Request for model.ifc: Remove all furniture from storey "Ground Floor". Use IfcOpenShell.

First a look at what the model holds.

```python
import ifcopenshell
import ifcopenshell.util.element

model = ifcopenshell.open("model.ifc")
print(model.schema)
storey = next(s for s in model.by_type("IfcBuildingStorey") if s.Name == "Ground Floor")
furniture = [e for e in ifcopenshell.util.element.get_decomposition(storey) if e.is_a("IfcFurnishingElement")]
seen = {}
for e in furniture:
    element_type = ifcopenshell.util.element.get_type(e)
    name = element_type.Name if element_type not in (None, e) else None
    seen[name] = seen.get(name, 0) + 1
for name, count in sorted(seen.items(), key=str):
    print(count, "x", name)
```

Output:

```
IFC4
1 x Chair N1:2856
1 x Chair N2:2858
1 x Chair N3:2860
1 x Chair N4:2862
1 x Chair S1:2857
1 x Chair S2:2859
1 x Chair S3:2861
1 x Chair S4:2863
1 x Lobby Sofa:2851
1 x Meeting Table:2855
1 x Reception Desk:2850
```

```python
import ifcopenshell
import ifcopenshell.api.root
import ifcopenshell.util.element

model = ifcopenshell.open("model.ifc")

storey = next(s for s in model.by_type("IfcBuildingStorey") if s.Name == "Ground Floor")
furniture = [e for e in ifcopenshell.util.element.get_decomposition(storey) if e.is_a("IfcFurnishingElement")]

for e in furniture:
    ifcopenshell.api.root.remove_product(model, product=e)
print(len(furniture), "removed")

model.write("model-out.ifc")
```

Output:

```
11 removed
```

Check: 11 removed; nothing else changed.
